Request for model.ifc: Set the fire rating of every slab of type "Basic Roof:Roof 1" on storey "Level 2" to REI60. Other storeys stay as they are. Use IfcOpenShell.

First a look at what the model holds.

```python
import ifcopenshell
import ifcopenshell.util.element

model = ifcopenshell.open("model.ifc")
print(model.schema)
storey = next(s for s in model.by_type("IfcBuildingStorey") if s.Name == "Level 2")
slabs = [e for e in ifcopenshell.util.element.get_decomposition(storey) if e.is_a("IfcSlab")]
seen = {}
for e in slabs:
    element_type = ifcopenshell.util.element.get_type(e)
    key = (element_type.Name if element_type != e and element_type else None, ifcopenshell.util.element.get_pset(e, "Pset_SlabCommon", "FireRating"))
    seen[key] = seen.get(key, 0) + 1
for (name, value), count in sorted(seen.items(), key=str):
    print(count, "x", name, "|", value)
```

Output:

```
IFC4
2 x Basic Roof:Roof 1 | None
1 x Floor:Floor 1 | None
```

```python
import ifcopenshell
import ifcopenshell.api.pset
import ifcopenshell.util.element

model = ifcopenshell.open("model.ifc")

storey = next(s for s in model.by_type("IfcBuildingStorey") if s.Name == "Level 2")
slabs = [e for e in ifcopenshell.util.element.get_decomposition(storey) if e.is_a("IfcSlab")]

count = 0
for e in slabs:
    element_type = ifcopenshell.util.element.get_type(e)
    if element_type in (None, e) or element_type.Name != "Basic Roof:Roof 1":
        continue
    # add_pset returns the element's existing set when there is one.
    pset = ifcopenshell.api.pset.add_pset(model, product=e, name="Pset_SlabCommon")
    ifcopenshell.api.pset.edit_pset(model, pset=pset, properties={"FireRating": "REI60"})
    count += 1

print(count, "slabs updated")

model.write("model_v2.ifc")
```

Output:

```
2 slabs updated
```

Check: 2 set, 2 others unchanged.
